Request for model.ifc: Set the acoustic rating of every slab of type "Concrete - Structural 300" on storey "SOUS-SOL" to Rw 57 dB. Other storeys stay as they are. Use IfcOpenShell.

First a look at what the model holds.

```python
import ifcopenshell
import ifcopenshell.util.element

model = ifcopenshell.open("model.ifc")
print(model.schema)
storey = next(s for s in model.by_type("IfcBuildingStorey") if s.Name == "SOUS-SOL")
slabs = [e for e in ifcopenshell.util.element.get_decomposition(storey) if e.is_a("IfcSlab")]
seen = {}
for e in slabs:
    element_type = ifcopenshell.util.element.get_type(e)
    key = (element_type.Name if element_type != e and element_type else None, ifcopenshell.util.element.get_pset(e, "Pset_SlabCommon", "AcousticRating"))
    seen[key] = seen.get(key, 0) + 1
for (name, value), count in sorted(seen.items(), key=str):
    print(count, "x", name, "|", value)
```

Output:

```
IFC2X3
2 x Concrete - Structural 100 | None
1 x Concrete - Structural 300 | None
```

```python
import ifcopenshell
import ifcopenshell.api.pset
import ifcopenshell.util.element

model = ifcopenshell.open("model.ifc")

storey = next(s for s in model.by_type("IfcBuildingStorey") if s.Name == "SOUS-SOL")
slabs = [e for e in ifcopenshell.util.element.get_decomposition(storey) if e.is_a("IfcSlab")]

count = 0
for e in slabs:
    element_type = ifcopenshell.util.element.get_type(e)
    if element_type in (None, e) or element_type.Name != "Concrete - Structural 300":
        continue
    # add_pset returns the element's existing set when there is one.
    pset = ifcopenshell.api.pset.add_pset(model, product=e, name="Pset_SlabCommon")
    ifcopenshell.api.pset.edit_pset(model, pset=pset, properties={"AcousticRating": "Rw 57 dB"})
    count += 1

print(count, "slabs updated")

model.write("model_edited.ifc")
```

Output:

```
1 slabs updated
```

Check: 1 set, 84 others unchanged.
